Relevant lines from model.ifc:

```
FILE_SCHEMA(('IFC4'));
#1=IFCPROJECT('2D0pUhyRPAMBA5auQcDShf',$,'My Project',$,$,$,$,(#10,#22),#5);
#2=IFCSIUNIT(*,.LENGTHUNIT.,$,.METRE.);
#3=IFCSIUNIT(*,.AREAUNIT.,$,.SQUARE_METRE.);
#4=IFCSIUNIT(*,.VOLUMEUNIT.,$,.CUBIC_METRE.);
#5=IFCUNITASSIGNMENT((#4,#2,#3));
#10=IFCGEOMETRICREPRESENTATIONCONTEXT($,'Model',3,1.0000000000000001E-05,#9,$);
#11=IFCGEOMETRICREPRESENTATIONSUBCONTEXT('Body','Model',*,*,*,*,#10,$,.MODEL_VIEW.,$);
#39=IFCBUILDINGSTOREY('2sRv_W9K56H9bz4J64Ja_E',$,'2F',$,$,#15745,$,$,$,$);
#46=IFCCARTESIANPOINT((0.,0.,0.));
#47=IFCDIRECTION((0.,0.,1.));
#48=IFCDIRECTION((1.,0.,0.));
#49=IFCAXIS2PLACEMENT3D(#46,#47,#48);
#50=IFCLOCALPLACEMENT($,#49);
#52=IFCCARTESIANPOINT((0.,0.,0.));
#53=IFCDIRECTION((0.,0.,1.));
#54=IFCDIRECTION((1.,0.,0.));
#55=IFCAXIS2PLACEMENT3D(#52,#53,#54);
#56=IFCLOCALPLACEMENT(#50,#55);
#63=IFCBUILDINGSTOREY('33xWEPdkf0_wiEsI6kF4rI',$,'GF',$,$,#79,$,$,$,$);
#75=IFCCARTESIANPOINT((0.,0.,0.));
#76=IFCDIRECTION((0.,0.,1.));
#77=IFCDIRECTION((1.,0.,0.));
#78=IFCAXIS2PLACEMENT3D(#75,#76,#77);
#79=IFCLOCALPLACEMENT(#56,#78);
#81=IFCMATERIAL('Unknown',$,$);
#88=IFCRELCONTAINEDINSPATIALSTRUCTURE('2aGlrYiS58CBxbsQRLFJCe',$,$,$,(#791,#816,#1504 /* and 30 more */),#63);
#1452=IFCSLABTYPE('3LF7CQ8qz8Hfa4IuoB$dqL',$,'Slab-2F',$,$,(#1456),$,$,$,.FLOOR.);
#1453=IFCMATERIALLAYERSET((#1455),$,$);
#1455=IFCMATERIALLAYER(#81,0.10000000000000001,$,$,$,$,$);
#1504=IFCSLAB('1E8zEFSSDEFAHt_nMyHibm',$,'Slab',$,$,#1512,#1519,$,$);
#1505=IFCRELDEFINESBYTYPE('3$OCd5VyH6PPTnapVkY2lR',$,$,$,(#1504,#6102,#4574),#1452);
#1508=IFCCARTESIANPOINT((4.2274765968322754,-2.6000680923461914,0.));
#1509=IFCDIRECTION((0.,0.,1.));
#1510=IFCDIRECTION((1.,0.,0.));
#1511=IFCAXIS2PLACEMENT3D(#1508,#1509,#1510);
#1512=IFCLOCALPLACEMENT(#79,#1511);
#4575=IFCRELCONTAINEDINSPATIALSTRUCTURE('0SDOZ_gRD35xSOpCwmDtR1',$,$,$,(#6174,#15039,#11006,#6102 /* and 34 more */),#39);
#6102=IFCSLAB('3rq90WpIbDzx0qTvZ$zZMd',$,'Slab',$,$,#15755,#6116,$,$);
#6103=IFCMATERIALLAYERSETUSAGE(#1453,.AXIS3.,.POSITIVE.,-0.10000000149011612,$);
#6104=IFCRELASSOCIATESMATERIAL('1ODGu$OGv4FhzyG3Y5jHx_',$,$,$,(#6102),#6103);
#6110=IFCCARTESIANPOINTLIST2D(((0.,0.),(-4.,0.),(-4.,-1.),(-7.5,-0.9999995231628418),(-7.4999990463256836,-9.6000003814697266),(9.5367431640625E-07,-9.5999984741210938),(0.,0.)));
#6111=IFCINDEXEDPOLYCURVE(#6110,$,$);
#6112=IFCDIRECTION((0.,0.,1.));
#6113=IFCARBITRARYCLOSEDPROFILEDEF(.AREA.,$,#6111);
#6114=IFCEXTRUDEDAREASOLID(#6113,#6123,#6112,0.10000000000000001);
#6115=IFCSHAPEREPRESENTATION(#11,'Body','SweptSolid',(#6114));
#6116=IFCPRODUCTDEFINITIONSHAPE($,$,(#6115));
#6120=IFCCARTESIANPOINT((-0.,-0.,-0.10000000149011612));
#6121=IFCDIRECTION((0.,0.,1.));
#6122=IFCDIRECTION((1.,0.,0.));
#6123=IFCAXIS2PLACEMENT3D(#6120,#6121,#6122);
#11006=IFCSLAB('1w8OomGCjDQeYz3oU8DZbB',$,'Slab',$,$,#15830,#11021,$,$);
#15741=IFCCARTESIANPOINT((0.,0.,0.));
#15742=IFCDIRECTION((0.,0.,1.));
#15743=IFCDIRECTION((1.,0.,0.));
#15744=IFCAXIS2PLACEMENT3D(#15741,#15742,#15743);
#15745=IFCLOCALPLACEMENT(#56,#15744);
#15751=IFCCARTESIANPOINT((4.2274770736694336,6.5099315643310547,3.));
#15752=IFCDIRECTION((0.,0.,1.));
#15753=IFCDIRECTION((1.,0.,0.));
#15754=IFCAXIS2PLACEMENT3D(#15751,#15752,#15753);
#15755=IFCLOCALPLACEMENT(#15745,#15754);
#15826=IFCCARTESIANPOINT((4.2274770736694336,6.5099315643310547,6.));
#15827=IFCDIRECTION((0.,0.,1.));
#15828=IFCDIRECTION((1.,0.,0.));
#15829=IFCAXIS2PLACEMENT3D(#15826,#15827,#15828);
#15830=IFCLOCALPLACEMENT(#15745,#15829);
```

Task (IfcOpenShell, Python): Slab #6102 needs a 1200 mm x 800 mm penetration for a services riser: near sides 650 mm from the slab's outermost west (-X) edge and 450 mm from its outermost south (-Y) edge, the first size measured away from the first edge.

```python
import numpy as np
import ifcopenshell
import ifcopenshell.api.feature
import ifcopenshell.api.geometry
import ifcopenshell.api.root
import ifcopenshell.geom
import ifcopenshell.util.placement
import ifcopenshell.util.representation
import ifcopenshell.util.shape
import ifcopenshell.util.unit

model = ifcopenshell.open("model.ifc")
unit_scale = ifcopenshell.util.unit.calculate_unit_scale(model)
settings = ifcopenshell.geom.settings()


def volume(element):
    """Net volume in cubic metres, openings subtracted."""
    shape = ifcopenshell.geom.create_shape(settings, element)
    return ifcopenshell.util.shape.get_volume(shape.geometry)


slab = model.by_guid("3rq90WpIbDzx0qTvZ$zZMd")
before = volume(slab)

# Extent in the slab's own axes, in metres. The edges named are its -X and -Y sides.
slab_shape = ifcopenshell.geom.create_shape(settings, slab)
vertices = ifcopenshell.util.shape.get_vertices(slab_shape.geometry)
x_min, y_min, bottom = vertices.min(axis=0)
top = vertices[:, 2].max()

opening = ifcopenshell.api.root.create_entity(model, ifc_class="IfcOpeningElement", name="Services riser opening", predefined_type="OPENING")
context = ifcopenshell.util.representation.get_context(model, "Model", "Body", "MODEL_VIEW")
width, depth = 1.2, 0.8
outline = [(0.0, 0.0), (width, 0.0), (width, depth), (0.0, depth), (0.0, 0.0)]
# Overshoot both faces by 50 mm so the cut is clean.
shape = ifcopenshell.api.geometry.add_slab_representation(
    model, context=context, depth=top - bottom + 0.1, polyline=outline
)
ifcopenshell.api.geometry.assign_representation(model, product=opening, representation=shape)

matrix = ifcopenshell.util.placement.get_local_placement(slab.ObjectPlacement)
matrix[:, 3] = matrix @ np.append(np.array([x_min + 0.65, y_min + 0.45, bottom - 0.05]) / unit_scale, 1.0)
ifcopenshell.api.geometry.edit_object_placement(model, product=opening, matrix=matrix, is_si=False)
ifcopenshell.api.feature.add_feature(model, feature=opening, element=slab)

after = volume(slab)

print(f"slab volume {before:.3f} -> {after:.3f} m3")

model.write("model-out.ifc")
```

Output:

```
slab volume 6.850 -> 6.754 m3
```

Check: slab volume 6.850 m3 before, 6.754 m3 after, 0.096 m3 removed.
